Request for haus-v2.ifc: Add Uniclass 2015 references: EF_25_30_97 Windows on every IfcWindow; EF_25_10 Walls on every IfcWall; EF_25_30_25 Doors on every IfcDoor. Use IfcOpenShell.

First a look at what the model holds.

```python
import ifcopenshell

model = ifcopenshell.open("haus-v2.ifc")
print(model.schema)
print("classifications:", [c.Name for c in model.by_type("IfcClassification")])
for ifc_class in ("IfcDoor", "IfcRoof", "IfcStair", "IfcWall", "IfcWindow"):
    print(ifc_class, len(model.by_type(ifc_class)))
```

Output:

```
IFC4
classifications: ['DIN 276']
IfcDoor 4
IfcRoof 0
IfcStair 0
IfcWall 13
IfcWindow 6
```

```python
import ifcopenshell
import ifcopenshell.api.classification

model = ifcopenshell.open("haus-v2.ifc")

system = ifcopenshell.api.classification.add_classification(model, classification="Uniclass 2015")

codes = {
    "IfcWindow": ("EF_25_30_97", "Windows"),
    "IfcWall": ("EF_25_10", "Walls"),
    "IfcDoor": ("EF_25_30_25", "Doors"),
}
for ifc_class, (code, name) in codes.items():
    products = model.by_type(ifc_class)
    ifcopenshell.api.classification.add_reference(
        model, products=products, classification=system, identification=code, name=name
    )
    print(code, len(products))

model.write("haus-v2_updated.ifc")
```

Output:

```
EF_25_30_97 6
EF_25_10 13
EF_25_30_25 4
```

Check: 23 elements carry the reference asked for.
